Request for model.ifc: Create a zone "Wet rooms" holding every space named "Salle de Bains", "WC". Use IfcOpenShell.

First a look at what the model holds.

```python
import ifcopenshell

model = ifcopenshell.open("model.ifc")
print(model.schema)
seen = {}
for space in model.by_type("IfcSpace"):
    seen[space.LongName] = seen.get(space.LongName, 0) + 1
for name, count in sorted(seen.items(), key=str):
    print(count, "x", name)
print("zones:", [z.Name for z in model.by_type("IfcZone")][:20])
```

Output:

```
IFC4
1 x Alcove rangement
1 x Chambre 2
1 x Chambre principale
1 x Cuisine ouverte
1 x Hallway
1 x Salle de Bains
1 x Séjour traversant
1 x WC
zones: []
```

```python
import ifcopenshell
import ifcopenshell.api.group
import ifcopenshell.api.root

model = ifcopenshell.open("model.ifc")

names = {"Salle de Bains", "WC"}
spaces = [s for s in model.by_type("IfcSpace") if s.LongName in names]

zone = ifcopenshell.api.root.create_entity(model, ifc_class="IfcZone", name="Wet rooms")
ifcopenshell.api.group.assign_group(model, products=spaces, group=zone)
print(len(spaces), "spaces in", zone.Name)

model.write("model_updated.ifc")
```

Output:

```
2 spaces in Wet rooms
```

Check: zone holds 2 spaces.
